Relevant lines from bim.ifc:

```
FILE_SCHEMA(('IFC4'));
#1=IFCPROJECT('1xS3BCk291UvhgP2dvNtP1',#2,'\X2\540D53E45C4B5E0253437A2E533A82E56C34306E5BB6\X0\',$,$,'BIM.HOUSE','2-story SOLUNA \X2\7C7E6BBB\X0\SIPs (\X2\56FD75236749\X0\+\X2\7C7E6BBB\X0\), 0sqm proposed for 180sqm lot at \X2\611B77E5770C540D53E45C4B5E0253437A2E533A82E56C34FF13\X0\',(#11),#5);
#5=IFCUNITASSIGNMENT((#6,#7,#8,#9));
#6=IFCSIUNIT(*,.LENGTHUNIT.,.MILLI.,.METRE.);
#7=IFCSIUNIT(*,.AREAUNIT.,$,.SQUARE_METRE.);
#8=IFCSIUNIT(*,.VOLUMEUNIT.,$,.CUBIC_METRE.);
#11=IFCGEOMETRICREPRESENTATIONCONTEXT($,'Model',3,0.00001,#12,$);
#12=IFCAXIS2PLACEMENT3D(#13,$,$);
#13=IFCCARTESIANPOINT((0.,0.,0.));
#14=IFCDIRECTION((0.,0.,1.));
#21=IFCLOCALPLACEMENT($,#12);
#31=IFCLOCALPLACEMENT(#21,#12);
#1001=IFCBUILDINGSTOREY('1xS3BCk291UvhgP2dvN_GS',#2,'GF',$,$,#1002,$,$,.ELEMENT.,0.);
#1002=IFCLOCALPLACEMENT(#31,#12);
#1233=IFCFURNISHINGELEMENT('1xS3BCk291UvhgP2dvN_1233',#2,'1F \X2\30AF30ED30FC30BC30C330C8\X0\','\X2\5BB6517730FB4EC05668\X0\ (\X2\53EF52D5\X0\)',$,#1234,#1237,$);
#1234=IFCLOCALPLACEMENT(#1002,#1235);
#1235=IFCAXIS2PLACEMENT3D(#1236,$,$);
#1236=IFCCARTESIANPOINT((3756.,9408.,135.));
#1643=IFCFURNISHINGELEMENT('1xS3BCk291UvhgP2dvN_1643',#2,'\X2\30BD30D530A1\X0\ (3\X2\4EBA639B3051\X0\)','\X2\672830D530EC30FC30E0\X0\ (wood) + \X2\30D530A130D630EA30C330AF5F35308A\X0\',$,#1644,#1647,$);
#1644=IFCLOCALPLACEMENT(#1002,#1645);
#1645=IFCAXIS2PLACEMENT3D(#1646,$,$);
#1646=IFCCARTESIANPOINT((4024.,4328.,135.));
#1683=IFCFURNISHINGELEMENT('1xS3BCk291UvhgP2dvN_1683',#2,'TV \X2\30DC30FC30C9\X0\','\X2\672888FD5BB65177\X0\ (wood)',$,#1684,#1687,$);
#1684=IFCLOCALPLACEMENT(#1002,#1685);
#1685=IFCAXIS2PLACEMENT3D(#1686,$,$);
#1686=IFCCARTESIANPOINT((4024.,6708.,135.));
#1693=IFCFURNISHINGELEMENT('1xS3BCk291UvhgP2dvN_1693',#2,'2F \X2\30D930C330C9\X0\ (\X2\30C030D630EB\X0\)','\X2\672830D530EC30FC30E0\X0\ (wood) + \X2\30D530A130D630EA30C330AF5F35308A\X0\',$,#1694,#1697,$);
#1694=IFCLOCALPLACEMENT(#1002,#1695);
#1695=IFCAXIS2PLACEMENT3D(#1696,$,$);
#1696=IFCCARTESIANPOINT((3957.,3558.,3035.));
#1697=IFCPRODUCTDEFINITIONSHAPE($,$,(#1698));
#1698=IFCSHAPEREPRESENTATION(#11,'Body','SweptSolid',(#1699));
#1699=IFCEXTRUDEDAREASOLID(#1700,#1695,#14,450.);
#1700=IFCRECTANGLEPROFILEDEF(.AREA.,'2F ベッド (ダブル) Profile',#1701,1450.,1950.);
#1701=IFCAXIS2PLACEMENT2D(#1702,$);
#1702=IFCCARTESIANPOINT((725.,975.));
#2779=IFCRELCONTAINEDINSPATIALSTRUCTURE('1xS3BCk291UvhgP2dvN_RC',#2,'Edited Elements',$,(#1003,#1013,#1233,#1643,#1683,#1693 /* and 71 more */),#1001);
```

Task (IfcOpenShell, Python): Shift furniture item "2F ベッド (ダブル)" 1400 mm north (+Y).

```python
import ifcopenshell
import ifcopenshell.api.geometry
import ifcopenshell.util.placement

model = ifcopenshell.open("bim.ifc")

item = model.by_guid("1xS3BCk291UvhgP2dvN_1693")
matrix = ifcopenshell.util.placement.get_local_placement(item.ObjectPlacement)
matrix[1, 3] += 1400.0
ifcopenshell.api.geometry.edit_object_placement(model, product=item, matrix=matrix, is_si=False)

print(ifcopenshell.util.placement.get_local_placement(item.ObjectPlacement).round(3) + 0.0)

model.write("bim_v2.ifc")
```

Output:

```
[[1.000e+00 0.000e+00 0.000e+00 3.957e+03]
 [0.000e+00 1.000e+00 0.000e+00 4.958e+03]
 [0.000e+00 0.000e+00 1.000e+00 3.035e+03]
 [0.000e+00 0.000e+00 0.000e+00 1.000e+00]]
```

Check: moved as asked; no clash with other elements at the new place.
